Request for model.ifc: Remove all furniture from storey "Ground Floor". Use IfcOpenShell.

First a look at what the model holds.

```python
import ifcopenshell
import ifcopenshell.util.element

model = ifcopenshell.open("model.ifc")
print(model.schema)
storey = next(s for s in model.by_type("IfcBuildingStorey") if s.Name == "Ground Floor")
furniture = [e for e in ifcopenshell.util.element.get_decomposition(storey) if e.is_a("IfcFurnishingElement")]
seen = {}
for e in furniture:
    element_type = ifcopenshell.util.element.get_type(e)
    name = element_type.Name if element_type not in (None, e) else None
    seen[name] = seen.get(name, 0) + 1
for name, count in sorted(seen.items(), key=str):
    print(count, "x", name)
```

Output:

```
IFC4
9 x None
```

```python
import ifcopenshell
import ifcopenshell.api.root
import ifcopenshell.util.element

model = ifcopenshell.open("model.ifc")

storey = next(s for s in model.by_type("IfcBuildingStorey") if s.Name == "Ground Floor")
furniture = [e for e in ifcopenshell.util.element.get_decomposition(storey) if e.is_a("IfcFurnishingElement")]

for e in furniture:
    ifcopenshell.api.root.remove_product(model, product=e)
print(len(furniture), "removed")

model.write("model_rev.ifc")
```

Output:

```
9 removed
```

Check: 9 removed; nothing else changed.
